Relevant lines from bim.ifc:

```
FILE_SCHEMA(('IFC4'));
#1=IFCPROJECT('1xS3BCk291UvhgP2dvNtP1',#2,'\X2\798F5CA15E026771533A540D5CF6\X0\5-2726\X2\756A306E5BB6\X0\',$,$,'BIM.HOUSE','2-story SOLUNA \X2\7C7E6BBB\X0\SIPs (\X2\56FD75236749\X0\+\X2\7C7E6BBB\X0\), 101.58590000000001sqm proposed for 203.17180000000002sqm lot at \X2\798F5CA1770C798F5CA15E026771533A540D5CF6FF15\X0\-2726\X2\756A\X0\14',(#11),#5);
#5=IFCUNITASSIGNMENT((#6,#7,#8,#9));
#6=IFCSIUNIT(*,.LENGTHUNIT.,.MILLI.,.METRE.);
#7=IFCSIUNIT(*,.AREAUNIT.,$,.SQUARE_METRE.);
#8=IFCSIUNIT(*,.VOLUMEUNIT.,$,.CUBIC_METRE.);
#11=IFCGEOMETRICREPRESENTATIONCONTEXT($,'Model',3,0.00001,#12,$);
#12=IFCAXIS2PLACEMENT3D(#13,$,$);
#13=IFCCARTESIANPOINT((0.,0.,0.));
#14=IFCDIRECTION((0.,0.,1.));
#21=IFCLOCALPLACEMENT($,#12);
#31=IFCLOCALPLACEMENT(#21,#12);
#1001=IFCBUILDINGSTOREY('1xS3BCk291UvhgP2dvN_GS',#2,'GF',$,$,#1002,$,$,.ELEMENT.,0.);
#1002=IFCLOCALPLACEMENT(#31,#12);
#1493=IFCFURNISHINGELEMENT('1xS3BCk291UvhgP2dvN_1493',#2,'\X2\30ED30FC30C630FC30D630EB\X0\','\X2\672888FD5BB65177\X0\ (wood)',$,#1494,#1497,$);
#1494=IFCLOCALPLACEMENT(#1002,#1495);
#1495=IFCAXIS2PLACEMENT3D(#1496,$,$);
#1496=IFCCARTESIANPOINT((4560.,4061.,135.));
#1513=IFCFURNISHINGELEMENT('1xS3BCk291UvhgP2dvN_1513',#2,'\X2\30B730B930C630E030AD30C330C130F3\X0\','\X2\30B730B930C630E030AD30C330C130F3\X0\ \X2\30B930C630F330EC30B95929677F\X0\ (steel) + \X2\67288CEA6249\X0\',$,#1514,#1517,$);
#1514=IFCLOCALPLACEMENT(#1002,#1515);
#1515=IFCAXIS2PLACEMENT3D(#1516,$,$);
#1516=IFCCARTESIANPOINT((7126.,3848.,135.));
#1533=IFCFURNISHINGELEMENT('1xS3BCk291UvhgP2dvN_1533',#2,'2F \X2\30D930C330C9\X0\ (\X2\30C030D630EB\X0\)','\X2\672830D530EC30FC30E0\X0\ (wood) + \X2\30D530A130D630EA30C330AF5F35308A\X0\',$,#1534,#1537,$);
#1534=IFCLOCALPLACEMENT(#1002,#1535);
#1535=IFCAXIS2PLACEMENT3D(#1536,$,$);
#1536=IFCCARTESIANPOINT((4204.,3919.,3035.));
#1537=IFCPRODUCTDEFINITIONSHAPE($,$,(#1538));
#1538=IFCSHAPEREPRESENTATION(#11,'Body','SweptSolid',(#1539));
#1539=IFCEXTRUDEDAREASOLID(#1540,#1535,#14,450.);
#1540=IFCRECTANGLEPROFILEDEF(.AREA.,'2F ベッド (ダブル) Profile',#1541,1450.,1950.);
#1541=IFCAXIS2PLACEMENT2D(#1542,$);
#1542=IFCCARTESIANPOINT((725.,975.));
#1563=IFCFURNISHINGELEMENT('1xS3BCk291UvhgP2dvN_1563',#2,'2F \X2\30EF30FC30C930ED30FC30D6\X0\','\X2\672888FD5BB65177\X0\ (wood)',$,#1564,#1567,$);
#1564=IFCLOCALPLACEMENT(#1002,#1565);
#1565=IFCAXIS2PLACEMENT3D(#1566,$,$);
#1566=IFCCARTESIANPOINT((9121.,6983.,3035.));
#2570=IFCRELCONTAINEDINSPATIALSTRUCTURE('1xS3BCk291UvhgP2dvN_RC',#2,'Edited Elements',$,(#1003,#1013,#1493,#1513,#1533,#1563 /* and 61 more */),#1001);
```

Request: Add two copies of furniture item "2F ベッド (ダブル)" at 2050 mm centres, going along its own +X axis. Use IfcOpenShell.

```python
import ifcopenshell
import ifcopenshell.api.geometry
import ifcopenshell.api.root
import ifcopenshell.util.element
import ifcopenshell.util.placement

model = ifcopenshell.open("bim.ifc")


def reuse_history(source, copy):
    """copy_class also copies each property set's owner history, people and application; keep the originals."""
    for rel in copy.IsDefinedBy:
        if rel.is_a("IfcRelDefinesByProperties") and (history := rel.RelatingPropertyDefinition.OwnerHistory):
            rel.RelatingPropertyDefinition.OwnerHistory = source.OwnerHistory
            ifcopenshell.util.element.remove_deep2(model, history)


source = model.by_id(1533)
base = ifcopenshell.util.placement.get_local_placement(source.ObjectPlacement)
step = base[:3, 0] * 2050.0

for i in range(1, 3):
    copy = ifcopenshell.api.root.copy_class(model, product=source)
    copy.Representation = ifcopenshell.util.element.copy_deep(
        model, source.Representation, exclude=["IfcGeometricRepresentationContext", "IfcRepresentationMap"]
    )
    reuse_history(source, copy)
    matrix = base.copy()
    matrix[:3, 3] += i * step
    print("added at", matrix[:3, 3].round(3) + 0.0)
    ifcopenshell.api.geometry.edit_object_placement(model, product=copy, matrix=matrix, is_si=False)

model.write("bim_v2.ifc")
```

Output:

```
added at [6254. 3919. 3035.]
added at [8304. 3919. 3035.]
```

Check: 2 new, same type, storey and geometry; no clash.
